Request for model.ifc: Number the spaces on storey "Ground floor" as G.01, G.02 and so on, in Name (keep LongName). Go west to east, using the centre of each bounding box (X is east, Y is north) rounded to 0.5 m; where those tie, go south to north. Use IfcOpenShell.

First a look at what the model holds.

```python
import ifcopenshell
import ifcopenshell.util.element
import ifcopenshell.util.placement

model = ifcopenshell.open("model.ifc")
print(model.schema)
storey = next(s for s in model.by_type("IfcBuildingStorey") if s.Name == "Ground floor")
spaces = [e for e in ifcopenshell.util.element.get_decomposition(storey) if e.is_a("IfcSpace")]
for e in sorted(spaces, key=lambda e: e.id()):
    origin = ifcopenshell.util.placement.get_local_placement(e.ObjectPlacement)[:3, 3]
    print(e.id(), e.Name, e.LongName, origin.round(2) + 0.0, sep=" | ")
```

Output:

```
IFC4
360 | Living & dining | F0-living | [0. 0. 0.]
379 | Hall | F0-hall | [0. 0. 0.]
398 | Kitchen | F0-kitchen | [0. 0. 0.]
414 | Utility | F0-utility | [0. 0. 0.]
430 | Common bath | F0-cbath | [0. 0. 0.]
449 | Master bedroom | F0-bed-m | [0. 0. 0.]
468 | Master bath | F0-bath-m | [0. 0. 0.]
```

```python
import ifcopenshell
import ifcopenshell.geom
import ifcopenshell.util.element
import ifcopenshell.util.shape

model = ifcopenshell.open("model.ifc")
settings = ifcopenshell.geom.settings()
settings.set("use-world-coords", True)


def centre(element):
    shape = ifcopenshell.geom.create_shape(settings, element)
    return ifcopenshell.util.shape.get_bbox_centroid(shape.geometry)


storey = next(s for s in model.by_type("IfcBuildingStorey") if s.Name == "Ground floor")
spaces = [e for e in ifcopenshell.util.element.get_decomposition(storey) if e.is_a("IfcSpace")]

# Insertion points can sit at a corner or the storey origin, so sort by the geometry (in metres).
centres = {e: centre(e) for e in spaces}
spaces.sort(key=lambda e: (round(centres[e][0] / 0.5), centres[e][1]))

for i, e in enumerate(spaces, start=1):
    number = f"G.{i:02d}"
    e.Name = number
    print(e.id(), number)

model.write("model_edited.ifc")
```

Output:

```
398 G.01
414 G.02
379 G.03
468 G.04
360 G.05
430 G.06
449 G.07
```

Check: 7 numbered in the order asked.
